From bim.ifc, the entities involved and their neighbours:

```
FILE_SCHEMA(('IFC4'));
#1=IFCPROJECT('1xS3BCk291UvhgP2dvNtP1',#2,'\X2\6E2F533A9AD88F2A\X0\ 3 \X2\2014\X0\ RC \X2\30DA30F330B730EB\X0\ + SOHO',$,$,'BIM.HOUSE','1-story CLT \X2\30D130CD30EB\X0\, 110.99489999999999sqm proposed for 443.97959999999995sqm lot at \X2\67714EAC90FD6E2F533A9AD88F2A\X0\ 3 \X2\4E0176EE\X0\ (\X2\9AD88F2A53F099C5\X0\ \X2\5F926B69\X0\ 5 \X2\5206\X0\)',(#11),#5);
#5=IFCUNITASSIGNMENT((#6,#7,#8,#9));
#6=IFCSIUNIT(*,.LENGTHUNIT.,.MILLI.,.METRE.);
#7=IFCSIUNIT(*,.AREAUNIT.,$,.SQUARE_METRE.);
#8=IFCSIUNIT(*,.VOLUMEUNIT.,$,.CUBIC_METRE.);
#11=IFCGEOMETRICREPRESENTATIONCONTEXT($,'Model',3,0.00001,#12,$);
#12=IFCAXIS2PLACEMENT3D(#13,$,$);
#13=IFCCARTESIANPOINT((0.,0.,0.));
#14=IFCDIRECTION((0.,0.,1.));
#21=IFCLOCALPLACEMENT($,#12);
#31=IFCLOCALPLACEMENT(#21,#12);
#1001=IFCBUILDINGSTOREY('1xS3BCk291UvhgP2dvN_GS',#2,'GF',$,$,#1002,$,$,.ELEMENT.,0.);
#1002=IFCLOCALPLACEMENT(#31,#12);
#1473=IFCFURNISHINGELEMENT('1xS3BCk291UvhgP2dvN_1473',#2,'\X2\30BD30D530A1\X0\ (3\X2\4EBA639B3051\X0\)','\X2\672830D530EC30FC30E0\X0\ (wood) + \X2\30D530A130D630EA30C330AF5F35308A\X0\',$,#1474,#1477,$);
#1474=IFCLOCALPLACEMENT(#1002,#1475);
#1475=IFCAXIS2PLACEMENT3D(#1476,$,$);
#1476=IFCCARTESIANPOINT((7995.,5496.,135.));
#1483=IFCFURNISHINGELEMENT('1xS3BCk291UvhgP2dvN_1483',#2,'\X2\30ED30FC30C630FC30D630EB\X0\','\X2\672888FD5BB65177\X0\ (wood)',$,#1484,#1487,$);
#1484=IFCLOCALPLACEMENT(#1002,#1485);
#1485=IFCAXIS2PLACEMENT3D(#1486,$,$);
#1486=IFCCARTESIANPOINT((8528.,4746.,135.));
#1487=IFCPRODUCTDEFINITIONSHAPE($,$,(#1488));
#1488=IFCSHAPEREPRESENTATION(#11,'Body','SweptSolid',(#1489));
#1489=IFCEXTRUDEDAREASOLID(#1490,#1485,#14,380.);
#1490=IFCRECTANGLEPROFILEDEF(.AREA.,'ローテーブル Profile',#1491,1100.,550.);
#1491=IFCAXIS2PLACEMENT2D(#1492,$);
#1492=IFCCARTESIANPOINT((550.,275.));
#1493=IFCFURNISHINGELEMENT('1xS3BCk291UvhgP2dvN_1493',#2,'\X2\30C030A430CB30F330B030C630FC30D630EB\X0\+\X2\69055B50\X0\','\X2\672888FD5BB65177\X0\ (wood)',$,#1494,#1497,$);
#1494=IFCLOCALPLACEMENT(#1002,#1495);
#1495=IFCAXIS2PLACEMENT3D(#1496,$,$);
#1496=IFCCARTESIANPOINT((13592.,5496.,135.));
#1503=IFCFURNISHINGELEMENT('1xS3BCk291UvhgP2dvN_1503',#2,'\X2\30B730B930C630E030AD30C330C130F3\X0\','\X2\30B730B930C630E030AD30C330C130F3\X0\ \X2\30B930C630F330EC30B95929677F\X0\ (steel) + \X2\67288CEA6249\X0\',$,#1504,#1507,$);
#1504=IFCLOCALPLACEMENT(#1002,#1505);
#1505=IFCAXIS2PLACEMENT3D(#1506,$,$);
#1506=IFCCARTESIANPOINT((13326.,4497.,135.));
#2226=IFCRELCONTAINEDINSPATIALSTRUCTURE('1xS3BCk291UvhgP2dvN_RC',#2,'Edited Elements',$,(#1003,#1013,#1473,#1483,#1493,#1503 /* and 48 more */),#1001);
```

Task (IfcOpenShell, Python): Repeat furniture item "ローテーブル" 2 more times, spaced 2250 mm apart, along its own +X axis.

```python
import ifcopenshell
import ifcopenshell.api.geometry
import ifcopenshell.api.root
import ifcopenshell.util.element
import ifcopenshell.util.placement

model = ifcopenshell.open("bim.ifc")


def reuse_history(source, copy):
    """copy_class also copies each property set's owner history, people and application; keep the originals."""
    for rel in copy.IsDefinedBy:
        if rel.is_a("IfcRelDefinesByProperties") and (history := rel.RelatingPropertyDefinition.OwnerHistory):
            rel.RelatingPropertyDefinition.OwnerHistory = source.OwnerHistory
            ifcopenshell.util.element.remove_deep2(model, history)


source = model.by_guid("1xS3BCk291UvhgP2dvN_1483")
base = ifcopenshell.util.placement.get_local_placement(source.ObjectPlacement)
step = base[:3, 0] * 2250.0

for i in range(1, 3):
    copy = ifcopenshell.api.root.copy_class(model, product=source)
    copy.Representation = ifcopenshell.util.element.copy_deep(
        model, source.Representation, exclude=["IfcGeometricRepresentationContext", "IfcRepresentationMap"]
    )
    reuse_history(source, copy)
    matrix = base.copy()
    matrix[:3, 3] += i * step
    print("added at", matrix[:3, 3].round(3) + 0.0)
    ifcopenshell.api.geometry.edit_object_placement(model, product=copy, matrix=matrix, is_si=False)

model.write("bim_rev.ifc")
```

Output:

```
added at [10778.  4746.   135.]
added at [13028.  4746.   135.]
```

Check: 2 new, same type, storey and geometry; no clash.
